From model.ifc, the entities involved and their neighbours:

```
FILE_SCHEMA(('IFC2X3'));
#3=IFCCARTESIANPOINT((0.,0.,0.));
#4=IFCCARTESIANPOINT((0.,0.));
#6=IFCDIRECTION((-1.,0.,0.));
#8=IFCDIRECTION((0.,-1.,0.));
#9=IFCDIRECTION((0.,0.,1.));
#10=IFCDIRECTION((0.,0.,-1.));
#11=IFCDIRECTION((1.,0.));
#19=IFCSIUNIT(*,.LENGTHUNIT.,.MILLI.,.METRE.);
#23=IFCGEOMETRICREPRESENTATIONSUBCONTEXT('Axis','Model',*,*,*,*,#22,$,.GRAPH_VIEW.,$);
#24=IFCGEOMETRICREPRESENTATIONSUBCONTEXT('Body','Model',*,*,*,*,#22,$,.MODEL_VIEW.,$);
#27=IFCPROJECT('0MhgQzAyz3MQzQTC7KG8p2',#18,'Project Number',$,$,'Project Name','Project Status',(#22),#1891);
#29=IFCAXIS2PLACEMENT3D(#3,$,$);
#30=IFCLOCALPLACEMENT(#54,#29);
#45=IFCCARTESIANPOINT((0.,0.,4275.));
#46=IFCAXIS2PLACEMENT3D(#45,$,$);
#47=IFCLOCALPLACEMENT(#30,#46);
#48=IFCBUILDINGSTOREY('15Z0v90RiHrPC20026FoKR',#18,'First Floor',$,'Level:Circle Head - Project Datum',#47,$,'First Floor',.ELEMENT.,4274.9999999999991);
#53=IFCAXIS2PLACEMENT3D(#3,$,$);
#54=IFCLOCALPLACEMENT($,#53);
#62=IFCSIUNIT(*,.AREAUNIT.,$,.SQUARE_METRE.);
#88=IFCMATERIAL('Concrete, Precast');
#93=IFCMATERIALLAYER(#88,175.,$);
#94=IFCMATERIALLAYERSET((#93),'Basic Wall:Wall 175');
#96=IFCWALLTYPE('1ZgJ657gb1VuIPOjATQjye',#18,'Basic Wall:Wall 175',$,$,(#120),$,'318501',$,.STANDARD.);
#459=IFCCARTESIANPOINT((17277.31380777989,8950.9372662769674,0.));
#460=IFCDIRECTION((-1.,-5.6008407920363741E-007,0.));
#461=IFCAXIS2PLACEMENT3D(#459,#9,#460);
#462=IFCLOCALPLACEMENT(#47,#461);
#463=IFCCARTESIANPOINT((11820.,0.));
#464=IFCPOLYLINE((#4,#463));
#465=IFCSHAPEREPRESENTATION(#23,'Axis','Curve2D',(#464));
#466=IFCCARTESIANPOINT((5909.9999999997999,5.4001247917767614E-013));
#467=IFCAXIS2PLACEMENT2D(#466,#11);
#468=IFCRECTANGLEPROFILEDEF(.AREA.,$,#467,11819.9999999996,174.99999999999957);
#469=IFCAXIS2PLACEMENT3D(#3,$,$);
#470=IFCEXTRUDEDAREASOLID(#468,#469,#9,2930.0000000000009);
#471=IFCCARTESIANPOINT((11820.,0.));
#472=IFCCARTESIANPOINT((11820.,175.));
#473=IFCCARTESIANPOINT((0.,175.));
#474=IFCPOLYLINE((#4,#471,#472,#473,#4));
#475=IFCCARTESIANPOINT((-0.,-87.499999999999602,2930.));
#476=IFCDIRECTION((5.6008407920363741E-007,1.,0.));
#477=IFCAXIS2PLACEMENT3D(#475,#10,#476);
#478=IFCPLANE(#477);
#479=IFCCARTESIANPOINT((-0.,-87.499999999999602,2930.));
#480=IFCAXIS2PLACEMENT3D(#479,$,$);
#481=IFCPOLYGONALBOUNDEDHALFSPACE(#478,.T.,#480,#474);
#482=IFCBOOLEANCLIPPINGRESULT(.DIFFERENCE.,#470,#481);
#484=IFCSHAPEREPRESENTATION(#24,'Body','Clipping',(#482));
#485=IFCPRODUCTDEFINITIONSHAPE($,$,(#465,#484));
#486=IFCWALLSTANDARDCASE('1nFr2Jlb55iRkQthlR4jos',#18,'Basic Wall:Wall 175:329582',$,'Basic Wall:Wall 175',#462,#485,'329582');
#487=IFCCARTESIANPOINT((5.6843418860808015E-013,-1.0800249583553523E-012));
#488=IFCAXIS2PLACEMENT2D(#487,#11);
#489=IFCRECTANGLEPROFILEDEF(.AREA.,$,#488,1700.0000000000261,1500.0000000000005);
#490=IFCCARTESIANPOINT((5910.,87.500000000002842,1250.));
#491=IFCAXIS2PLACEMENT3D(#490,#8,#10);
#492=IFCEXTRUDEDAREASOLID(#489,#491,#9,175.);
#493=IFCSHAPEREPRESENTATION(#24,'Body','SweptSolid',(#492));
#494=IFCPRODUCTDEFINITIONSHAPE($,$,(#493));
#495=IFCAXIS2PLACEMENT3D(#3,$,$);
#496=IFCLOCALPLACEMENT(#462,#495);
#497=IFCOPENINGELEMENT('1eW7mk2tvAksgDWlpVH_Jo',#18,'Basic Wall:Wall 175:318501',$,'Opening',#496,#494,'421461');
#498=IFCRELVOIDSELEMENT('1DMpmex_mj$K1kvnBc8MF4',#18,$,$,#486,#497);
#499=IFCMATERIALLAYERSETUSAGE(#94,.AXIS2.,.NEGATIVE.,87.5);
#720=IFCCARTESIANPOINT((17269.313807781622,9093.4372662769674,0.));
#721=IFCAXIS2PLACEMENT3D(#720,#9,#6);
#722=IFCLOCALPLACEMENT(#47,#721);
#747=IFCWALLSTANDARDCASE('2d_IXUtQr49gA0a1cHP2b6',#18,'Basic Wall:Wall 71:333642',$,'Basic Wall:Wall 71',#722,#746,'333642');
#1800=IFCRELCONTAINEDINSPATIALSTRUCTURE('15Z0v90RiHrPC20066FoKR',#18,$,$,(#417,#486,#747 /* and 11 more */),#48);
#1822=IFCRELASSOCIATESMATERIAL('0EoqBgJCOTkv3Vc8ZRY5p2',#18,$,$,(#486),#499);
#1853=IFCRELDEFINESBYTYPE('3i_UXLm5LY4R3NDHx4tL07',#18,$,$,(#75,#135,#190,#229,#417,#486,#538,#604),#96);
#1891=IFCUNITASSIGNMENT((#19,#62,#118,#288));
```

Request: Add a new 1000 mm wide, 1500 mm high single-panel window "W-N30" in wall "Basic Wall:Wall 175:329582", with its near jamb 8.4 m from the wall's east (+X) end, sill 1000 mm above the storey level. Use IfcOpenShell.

```python
import numpy as np
import ifcopenshell
import ifcopenshell.api.feature
import ifcopenshell.api.geometry
import ifcopenshell.api.root
import ifcopenshell.api.spatial
import ifcopenshell.api.type
import ifcopenshell.geom
import ifcopenshell.util.element
import ifcopenshell.util.placement
import ifcopenshell.util.representation
import ifcopenshell.util.shape
import ifcopenshell.util.unit

model = ifcopenshell.open("model.ifc")
unit_scale = ifcopenshell.util.unit.calculate_unit_scale(model)
settings = ifcopenshell.geom.settings()


def volume(element):
    """Net volume in cubic metres, openings subtracted."""
    shape = ifcopenshell.geom.create_shape(settings, element)
    return ifcopenshell.util.shape.get_volume(shape.geometry)


wall = model.by_guid("1nFr2Jlb55iRkQthlR4jos")
storey = ifcopenshell.util.element.get_container(wall, ifc_class="IfcBuildingStorey")
context = ifcopenshell.util.representation.get_context(model, "Model", "Body", "MODEL_VIEW")
before = volume(wall)

width, height, from_end, sill = 1, 1.5, 8.4, 1  # metres

# The wall runs along its own X axis, and the end named is its -X end.
wall_shape = ifcopenshell.geom.create_shape(settings, wall)
x, y, z = ifcopenshell.util.shape.get_vertices(wall_shape.geometry).T
start = x.min() + from_end
face, thickness = float(y.min()), float(y.max() - y.min())
wall_matrix = ifcopenshell.util.placement.get_local_placement(wall.ObjectPlacement)
level = ifcopenshell.util.placement.get_local_placement(storey.ObjectPlacement)[2, 3]


def in_wall(x, y):
    """Placement at x, y metres in the wall's axes, at sill height."""
    matrix = wall_matrix.copy()
    matrix[:, 3] = wall_matrix @ np.array([x / unit_scale, y / unit_scale, 0.0, 1.0])
    matrix[2, 3] = level + sill / unit_scale
    return matrix


# Opening: a box that overshoots both wall faces by 50 mm.
opening = ifcopenshell.api.root.create_entity(model, ifc_class="IfcOpeningElement")
box = ifcopenshell.api.geometry.add_wall_representation(
    model, context=context, length=width, height=height, thickness=thickness + 0.1
)
ifcopenshell.api.geometry.assign_representation(model, product=opening, representation=box)
ifcopenshell.api.geometry.edit_object_placement(model, product=opening, matrix=in_wall(start, face - 0.05), is_si=False)
ifcopenshell.api.feature.add_feature(model, feature=opening, element=wall)

window = ifcopenshell.api.root.create_entity(model, ifc_class="IfcWindow", name="W-N30")
window.OverallWidth, window.OverallHeight = width / unit_scale, height / unit_scale
body = ifcopenshell.api.geometry.add_window_representation(
    model,
    context=context,
    overall_width=window.OverallWidth,
    overall_height=window.OverallHeight,
    partition_type="SINGLE_PANEL",
)
ifcopenshell.api.geometry.assign_representation(model, product=window, representation=body)
ifcopenshell.api.spatial.assign_container(model, products=[window], relating_structure=storey)
fills = ifcopenshell.api.feature.add_filling(model, opening=opening, element=window)
fills.OwnerHistory = window.OwnerHistory  # required in IFC2X3

# IFC2X3 keeps the operation on the window style.
style = ifcopenshell.api.root.create_entity(model, ifc_class="IfcWindowStyle", name="W-N30")
style.OperationType, style.ConstructionType = "SINGLE_PANEL", "NOTDEFINED"
style.ParameterTakesPrecedence = style.Sizeable = False
ifcopenshell.api.type.assign_type(model, related_objects=[window], relating_type=style)

# Centre the window in the wall's thickness.
ifcopenshell.api.geometry.edit_object_placement(model, product=window, matrix=in_wall(start, face), is_si=False)
window_shape = ifcopenshell.geom.create_shape(settings, window)
depth = ifcopenshell.util.shape.get_vertices(window_shape.geometry)[:, 1]
offset = face + thickness / 2 - (depth.min() + depth.max()) / 2
ifcopenshell.api.geometry.edit_object_placement(model, product=window, matrix=in_wall(start, offset), is_si=False)

after = volume(wall)

print(f"wall volume {before:.3f} -> {after:.3f} m3")

model.write("model_updated.ifc")
```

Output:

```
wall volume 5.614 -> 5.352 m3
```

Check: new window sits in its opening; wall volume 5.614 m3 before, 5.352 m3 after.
